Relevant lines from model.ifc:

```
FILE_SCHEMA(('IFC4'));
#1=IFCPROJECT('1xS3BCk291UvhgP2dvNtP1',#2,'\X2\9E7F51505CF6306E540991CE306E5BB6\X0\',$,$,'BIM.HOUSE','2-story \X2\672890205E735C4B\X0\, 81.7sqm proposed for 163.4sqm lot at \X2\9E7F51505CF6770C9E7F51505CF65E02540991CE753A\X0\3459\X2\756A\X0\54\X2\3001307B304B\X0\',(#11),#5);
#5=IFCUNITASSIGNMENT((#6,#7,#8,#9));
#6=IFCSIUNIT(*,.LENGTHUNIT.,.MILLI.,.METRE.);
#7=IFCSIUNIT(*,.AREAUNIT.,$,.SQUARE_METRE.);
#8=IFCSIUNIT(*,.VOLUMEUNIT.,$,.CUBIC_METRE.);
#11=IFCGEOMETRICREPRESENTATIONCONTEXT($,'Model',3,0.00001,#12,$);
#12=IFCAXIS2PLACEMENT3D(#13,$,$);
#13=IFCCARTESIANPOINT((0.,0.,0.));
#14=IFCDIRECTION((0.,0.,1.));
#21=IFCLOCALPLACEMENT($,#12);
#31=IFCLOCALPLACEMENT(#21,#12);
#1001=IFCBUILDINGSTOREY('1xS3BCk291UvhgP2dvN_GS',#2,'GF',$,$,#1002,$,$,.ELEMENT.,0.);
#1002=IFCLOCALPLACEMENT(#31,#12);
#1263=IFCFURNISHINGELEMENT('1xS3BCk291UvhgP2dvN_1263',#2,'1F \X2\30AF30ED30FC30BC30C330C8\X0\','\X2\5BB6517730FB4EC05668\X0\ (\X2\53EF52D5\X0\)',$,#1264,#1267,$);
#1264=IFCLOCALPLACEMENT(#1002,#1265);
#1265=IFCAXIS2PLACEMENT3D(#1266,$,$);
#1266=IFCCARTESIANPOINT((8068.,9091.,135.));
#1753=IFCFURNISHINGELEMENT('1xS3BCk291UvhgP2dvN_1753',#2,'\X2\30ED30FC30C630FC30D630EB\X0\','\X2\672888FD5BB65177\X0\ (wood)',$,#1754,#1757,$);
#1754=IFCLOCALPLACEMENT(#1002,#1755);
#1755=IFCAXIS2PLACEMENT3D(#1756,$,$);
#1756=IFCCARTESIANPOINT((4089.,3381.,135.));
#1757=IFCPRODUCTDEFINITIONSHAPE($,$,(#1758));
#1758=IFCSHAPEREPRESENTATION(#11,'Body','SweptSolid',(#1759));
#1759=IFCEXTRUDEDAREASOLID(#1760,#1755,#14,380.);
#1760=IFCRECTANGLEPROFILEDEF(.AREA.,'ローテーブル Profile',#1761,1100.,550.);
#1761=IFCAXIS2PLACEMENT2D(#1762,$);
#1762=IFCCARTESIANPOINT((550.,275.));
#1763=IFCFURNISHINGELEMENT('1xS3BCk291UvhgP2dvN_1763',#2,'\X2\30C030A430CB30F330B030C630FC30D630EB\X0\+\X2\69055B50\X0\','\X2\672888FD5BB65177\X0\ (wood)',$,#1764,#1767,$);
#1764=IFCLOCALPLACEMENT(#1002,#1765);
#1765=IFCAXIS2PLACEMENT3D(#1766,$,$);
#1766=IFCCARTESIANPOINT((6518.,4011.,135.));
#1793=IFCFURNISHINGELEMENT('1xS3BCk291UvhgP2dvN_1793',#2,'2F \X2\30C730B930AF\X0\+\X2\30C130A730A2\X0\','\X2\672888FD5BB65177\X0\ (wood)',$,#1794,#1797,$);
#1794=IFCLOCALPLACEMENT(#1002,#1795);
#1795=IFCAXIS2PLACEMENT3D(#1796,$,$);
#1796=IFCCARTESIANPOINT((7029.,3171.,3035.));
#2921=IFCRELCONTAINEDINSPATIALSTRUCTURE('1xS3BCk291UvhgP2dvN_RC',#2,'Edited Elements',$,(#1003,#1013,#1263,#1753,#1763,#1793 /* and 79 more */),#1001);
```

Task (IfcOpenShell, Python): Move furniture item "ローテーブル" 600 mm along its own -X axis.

```python
import ifcopenshell
import ifcopenshell.api.geometry
import ifcopenshell.util.placement
import ifcopenshell.util.unit

model = ifcopenshell.open("model.ifc")
unit_scale = ifcopenshell.util.unit.calculate_unit_scale(model)

item = model.by_guid("1xS3BCk291UvhgP2dvN_1753")
matrix = ifcopenshell.util.placement.get_local_placement(item.ObjectPlacement)
matrix[:3, 3] -= matrix[:3, 0] * 0.6 / unit_scale
ifcopenshell.api.geometry.edit_object_placement(model, product=item, matrix=matrix, is_si=False)

print(ifcopenshell.util.placement.get_local_placement(item.ObjectPlacement).round(3) + 0.0)

model.write("model_updated.ifc")
```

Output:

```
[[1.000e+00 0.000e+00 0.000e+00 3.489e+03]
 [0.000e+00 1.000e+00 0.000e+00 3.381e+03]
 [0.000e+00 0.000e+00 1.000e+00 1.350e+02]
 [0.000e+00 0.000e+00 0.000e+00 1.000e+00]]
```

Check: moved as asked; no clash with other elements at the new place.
